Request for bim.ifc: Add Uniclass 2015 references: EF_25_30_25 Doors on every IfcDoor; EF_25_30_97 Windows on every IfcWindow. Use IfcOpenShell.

First a look at what the model holds.

```python
import ifcopenshell

model = ifcopenshell.open("bim.ifc")
print(model.schema)
print("classifications:", [c.Name for c in model.by_type("IfcClassification")])
for ifc_class in ("IfcDoor", "IfcRoof", "IfcStair", "IfcWall", "IfcWindow"):
    print(ifc_class, len(model.by_type(ifc_class)))
```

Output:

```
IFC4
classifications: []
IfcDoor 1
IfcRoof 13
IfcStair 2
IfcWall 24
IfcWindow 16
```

```python
import ifcopenshell
import ifcopenshell.api.classification

model = ifcopenshell.open("bim.ifc")

system = ifcopenshell.api.classification.add_classification(model, classification="Uniclass 2015")

codes = {
    "IfcDoor": ("EF_25_30_25", "Doors"),
    "IfcWindow": ("EF_25_30_97", "Windows"),
}
for ifc_class, (code, name) in codes.items():
    products = model.by_type(ifc_class)
    ifcopenshell.api.classification.add_reference(
        model, products=products, classification=system, identification=code, name=name
    )
    print(code, len(products))

model.write("bim_rev.ifc")
```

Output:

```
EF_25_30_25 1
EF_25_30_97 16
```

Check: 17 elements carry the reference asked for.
